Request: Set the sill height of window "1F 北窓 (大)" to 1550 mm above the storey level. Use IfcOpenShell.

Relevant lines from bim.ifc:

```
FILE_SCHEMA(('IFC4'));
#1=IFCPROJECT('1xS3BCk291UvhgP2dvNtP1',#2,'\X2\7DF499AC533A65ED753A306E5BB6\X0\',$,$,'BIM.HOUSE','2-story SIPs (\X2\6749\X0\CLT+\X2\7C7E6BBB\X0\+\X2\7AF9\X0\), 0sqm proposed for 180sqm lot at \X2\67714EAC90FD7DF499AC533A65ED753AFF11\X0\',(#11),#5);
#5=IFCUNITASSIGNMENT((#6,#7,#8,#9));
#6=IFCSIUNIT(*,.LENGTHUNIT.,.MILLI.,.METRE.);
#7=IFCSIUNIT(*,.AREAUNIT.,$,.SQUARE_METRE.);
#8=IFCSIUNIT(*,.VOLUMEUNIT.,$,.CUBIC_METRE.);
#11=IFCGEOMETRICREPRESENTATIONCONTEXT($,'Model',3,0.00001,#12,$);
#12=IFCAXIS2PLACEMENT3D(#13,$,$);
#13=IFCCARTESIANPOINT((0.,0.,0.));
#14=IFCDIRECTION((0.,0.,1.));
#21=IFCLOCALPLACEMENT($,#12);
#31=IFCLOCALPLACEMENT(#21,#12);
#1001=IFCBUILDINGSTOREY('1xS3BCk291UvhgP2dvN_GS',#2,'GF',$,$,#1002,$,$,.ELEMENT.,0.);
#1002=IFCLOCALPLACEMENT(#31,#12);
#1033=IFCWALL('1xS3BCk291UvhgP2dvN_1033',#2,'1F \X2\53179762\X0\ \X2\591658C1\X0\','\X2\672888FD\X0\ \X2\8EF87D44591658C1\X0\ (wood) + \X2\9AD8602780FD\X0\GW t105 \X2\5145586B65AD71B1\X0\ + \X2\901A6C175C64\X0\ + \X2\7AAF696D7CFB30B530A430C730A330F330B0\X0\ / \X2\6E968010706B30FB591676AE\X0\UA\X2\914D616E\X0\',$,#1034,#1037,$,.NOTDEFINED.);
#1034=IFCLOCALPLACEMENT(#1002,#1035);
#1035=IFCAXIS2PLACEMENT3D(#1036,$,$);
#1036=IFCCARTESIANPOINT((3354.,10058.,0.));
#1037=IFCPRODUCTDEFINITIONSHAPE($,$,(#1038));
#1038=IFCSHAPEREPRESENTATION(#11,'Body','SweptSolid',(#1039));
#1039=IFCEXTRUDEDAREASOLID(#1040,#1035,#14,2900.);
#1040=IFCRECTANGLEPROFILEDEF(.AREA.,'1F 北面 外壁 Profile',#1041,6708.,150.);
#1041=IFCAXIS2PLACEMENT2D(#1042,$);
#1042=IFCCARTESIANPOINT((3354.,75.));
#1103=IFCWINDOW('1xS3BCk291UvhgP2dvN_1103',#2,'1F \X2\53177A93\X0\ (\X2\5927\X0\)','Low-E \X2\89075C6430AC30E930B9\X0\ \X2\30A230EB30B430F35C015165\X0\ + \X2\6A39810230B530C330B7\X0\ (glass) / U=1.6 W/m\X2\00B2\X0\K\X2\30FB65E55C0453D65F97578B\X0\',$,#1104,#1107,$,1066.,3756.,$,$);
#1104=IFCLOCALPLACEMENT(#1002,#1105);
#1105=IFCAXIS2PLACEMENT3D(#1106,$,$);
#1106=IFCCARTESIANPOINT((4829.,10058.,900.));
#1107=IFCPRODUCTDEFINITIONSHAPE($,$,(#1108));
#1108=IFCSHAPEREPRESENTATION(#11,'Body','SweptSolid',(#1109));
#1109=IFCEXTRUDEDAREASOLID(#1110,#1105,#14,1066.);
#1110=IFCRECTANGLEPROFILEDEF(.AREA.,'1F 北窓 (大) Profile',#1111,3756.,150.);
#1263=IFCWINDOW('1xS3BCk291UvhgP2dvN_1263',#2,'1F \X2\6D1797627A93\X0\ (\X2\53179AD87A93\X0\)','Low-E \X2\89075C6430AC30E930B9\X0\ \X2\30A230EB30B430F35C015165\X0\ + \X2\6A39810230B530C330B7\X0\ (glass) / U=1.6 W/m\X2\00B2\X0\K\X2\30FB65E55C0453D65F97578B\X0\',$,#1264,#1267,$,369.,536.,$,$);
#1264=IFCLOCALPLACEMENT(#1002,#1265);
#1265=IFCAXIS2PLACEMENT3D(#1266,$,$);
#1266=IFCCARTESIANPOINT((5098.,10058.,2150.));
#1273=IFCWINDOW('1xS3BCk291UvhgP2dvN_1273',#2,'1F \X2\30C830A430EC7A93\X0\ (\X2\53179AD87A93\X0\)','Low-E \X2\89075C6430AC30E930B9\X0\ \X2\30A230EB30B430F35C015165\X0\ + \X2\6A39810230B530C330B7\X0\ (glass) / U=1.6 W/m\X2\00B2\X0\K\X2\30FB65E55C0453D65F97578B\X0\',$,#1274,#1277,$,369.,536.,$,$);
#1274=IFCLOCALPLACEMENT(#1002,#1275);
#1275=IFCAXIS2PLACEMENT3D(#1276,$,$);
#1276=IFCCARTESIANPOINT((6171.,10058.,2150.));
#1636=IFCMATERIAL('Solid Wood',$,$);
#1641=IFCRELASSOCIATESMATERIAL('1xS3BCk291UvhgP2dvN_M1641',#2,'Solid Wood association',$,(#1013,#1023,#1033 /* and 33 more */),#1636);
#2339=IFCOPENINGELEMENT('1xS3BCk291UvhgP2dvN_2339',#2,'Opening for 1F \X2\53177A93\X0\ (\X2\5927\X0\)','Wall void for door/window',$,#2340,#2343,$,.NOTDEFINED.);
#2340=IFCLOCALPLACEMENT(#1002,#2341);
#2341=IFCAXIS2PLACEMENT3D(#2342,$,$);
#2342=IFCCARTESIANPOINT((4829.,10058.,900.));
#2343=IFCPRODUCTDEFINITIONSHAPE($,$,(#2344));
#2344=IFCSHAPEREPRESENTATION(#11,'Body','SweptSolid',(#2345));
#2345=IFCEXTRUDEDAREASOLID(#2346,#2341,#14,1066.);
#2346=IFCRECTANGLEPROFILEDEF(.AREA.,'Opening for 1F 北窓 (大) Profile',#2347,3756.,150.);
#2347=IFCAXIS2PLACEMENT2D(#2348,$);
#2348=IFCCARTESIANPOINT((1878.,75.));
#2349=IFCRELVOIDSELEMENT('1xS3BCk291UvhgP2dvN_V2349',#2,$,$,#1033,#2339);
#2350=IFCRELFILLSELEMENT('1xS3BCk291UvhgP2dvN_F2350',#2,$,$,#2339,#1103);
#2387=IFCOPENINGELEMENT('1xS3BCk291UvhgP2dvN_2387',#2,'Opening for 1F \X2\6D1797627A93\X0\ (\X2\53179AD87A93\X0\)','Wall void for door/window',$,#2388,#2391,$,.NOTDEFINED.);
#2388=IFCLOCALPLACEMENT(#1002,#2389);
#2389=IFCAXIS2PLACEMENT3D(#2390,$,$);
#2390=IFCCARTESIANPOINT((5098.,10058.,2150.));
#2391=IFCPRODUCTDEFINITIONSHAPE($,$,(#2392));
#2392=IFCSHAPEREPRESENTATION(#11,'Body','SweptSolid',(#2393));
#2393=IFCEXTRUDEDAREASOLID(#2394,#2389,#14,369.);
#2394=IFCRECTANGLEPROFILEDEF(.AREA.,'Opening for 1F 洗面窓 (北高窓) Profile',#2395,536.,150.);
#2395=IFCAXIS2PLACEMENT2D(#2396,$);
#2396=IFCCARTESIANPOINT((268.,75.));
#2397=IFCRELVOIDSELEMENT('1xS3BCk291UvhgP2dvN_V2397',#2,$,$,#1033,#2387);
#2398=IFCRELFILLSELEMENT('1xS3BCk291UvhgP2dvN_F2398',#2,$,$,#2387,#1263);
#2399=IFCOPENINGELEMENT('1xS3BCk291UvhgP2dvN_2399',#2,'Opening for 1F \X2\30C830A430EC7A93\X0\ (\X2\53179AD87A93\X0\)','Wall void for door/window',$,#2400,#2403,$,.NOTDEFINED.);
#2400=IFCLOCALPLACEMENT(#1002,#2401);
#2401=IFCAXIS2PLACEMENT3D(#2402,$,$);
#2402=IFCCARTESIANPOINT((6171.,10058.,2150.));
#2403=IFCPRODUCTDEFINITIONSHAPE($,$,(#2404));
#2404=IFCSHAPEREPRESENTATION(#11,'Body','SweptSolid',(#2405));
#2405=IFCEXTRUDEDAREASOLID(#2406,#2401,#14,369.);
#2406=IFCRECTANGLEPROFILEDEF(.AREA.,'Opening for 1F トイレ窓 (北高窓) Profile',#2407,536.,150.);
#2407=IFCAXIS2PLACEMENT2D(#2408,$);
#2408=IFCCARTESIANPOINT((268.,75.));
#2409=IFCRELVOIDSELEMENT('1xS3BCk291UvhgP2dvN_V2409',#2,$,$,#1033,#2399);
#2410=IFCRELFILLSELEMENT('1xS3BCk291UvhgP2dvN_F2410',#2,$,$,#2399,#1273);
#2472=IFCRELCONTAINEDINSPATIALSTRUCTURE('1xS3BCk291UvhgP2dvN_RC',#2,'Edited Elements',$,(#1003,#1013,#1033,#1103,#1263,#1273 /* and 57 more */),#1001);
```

```python
import numpy as np
import ifcopenshell
import ifcopenshell.api.geometry
import ifcopenshell.geom
import ifcopenshell.util.element
import ifcopenshell.util.placement
import ifcopenshell.util.shape
import ifcopenshell.util.unit

model = ifcopenshell.open("bim.ifc")
unit_scale = ifcopenshell.util.unit.calculate_unit_scale(model)

window = model.by_guid("1xS3BCk291UvhgP2dvN_1103")
opening = window.FillsVoids[0].RelatingOpeningElement
storey = ifcopenshell.util.element.get_container(window, ifc_class="IfcBuildingStorey")
level = ifcopenshell.util.placement.get_local_placement(storey.ObjectPlacement)[2, 3]

# The opening's origin need not be at the sill, so measure its lowest point.
shape = ifcopenshell.geom.create_shape(ifcopenshell.geom.settings(), opening)
bottom = ifcopenshell.util.shape.get_shape_bottom_elevation(shape, shape.geometry) / unit_scale
dz = level + 1.55 / unit_scale - bottom

shift = np.array([0.0, 0.0, dz])
# The window is not placed relative to its opening, so move both.
for product in (opening, window):
    matrix = ifcopenshell.util.placement.get_local_placement(product.ObjectPlacement)
    matrix[:3, 3] += shift
    ifcopenshell.api.geometry.edit_object_placement(model, product=product, matrix=matrix, is_si=False)

print(f"moved by {dz * unit_scale:+.3f} m")

model.write("bim_rev.ifc")
```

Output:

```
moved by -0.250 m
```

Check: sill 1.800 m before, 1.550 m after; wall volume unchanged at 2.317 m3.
